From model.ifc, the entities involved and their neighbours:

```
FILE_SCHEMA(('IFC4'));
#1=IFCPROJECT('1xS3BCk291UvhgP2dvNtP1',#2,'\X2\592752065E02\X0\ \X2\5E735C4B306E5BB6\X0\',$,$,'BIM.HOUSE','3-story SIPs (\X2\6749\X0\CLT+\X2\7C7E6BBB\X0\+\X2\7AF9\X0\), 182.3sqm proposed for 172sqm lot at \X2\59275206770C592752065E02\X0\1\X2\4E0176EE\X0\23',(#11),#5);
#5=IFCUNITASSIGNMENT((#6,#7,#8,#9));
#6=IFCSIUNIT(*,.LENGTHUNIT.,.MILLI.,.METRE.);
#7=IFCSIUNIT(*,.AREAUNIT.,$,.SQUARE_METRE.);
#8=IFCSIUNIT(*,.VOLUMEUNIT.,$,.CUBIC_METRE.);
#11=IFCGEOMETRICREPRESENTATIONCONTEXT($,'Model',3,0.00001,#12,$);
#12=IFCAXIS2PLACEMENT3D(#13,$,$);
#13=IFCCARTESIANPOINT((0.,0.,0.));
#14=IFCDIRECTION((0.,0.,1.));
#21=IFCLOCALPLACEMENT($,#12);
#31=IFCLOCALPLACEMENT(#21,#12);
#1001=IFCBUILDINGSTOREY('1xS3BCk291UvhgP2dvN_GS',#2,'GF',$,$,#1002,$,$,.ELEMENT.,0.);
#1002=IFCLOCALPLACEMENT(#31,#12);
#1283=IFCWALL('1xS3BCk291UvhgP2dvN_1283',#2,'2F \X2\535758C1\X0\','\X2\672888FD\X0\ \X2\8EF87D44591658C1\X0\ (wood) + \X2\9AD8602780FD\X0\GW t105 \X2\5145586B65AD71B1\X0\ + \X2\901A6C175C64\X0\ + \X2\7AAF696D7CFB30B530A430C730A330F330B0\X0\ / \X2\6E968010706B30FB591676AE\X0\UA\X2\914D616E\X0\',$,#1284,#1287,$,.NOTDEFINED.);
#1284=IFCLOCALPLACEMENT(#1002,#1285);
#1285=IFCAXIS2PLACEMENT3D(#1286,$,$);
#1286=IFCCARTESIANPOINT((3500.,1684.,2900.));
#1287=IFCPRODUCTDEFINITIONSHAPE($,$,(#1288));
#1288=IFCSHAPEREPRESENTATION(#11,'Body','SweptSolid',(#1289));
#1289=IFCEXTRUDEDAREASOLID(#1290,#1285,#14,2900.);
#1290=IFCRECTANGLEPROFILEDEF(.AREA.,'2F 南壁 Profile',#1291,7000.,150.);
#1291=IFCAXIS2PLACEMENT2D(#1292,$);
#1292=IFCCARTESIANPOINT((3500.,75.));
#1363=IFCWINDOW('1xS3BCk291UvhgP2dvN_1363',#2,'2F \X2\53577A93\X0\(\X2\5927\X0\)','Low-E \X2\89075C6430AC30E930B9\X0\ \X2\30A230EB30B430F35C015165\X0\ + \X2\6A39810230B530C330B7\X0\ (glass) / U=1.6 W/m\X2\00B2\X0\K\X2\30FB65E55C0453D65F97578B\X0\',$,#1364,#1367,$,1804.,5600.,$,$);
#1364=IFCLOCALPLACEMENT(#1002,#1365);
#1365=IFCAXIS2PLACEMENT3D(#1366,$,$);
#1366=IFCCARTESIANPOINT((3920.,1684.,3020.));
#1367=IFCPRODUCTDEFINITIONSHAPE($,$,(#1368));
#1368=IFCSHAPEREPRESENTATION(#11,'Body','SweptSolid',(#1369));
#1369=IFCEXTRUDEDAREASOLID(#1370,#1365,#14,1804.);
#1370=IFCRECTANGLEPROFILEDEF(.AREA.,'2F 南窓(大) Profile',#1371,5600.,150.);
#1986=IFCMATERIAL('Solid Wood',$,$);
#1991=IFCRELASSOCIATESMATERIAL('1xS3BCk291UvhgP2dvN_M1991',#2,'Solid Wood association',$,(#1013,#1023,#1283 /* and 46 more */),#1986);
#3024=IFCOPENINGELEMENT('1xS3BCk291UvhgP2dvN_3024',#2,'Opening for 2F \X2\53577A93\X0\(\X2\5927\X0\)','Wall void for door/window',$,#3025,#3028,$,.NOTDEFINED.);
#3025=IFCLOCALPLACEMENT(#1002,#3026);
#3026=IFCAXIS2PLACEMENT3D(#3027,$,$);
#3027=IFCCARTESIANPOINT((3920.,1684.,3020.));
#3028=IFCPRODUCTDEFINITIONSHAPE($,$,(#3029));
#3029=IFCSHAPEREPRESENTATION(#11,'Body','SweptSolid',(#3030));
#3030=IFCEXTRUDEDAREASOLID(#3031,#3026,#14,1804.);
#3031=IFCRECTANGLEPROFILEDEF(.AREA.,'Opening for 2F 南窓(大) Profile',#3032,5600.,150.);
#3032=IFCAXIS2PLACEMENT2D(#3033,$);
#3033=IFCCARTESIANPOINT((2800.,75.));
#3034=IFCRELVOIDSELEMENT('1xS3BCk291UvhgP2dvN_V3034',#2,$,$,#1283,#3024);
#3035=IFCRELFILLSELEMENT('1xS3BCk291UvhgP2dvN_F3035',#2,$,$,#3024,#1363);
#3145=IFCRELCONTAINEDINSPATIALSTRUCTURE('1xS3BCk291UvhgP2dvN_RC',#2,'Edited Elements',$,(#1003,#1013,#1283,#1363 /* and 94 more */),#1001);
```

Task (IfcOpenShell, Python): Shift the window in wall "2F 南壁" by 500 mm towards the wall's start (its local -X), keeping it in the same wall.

```python
import ifcopenshell
import ifcopenshell.api.geometry
import ifcopenshell.util.placement

model = ifcopenshell.open("model.ifc")

window = model.by_guid("1xS3BCk291UvhgP2dvN_1363")
opening = window.FillsVoids[0].RelatingOpeningElement
wall = opening.VoidsElements[0].RelatingBuildingElement

wall_matrix = ifcopenshell.util.placement.get_local_placement(wall.ObjectPlacement)
shift = wall_matrix[:3, 0] * -500.0
before = ifcopenshell.util.placement.get_local_placement(window.ObjectPlacement)[:3, 3].copy()

# The window is not placed relative to its opening, so move both.
for product in (opening, window):
    matrix = ifcopenshell.util.placement.get_local_placement(product.ObjectPlacement)
    matrix[:3, 3] += shift
    ifcopenshell.api.geometry.edit_object_placement(model, product=product, matrix=matrix, is_si=False)

after = ifcopenshell.util.placement.get_local_placement(window.ObjectPlacement)[:3, 3]
print("window moved by", (after - before).round(3) + 0.0)

model.write("model_updated.ifc")
```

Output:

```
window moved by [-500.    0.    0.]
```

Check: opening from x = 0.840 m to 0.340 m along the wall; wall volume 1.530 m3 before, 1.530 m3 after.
